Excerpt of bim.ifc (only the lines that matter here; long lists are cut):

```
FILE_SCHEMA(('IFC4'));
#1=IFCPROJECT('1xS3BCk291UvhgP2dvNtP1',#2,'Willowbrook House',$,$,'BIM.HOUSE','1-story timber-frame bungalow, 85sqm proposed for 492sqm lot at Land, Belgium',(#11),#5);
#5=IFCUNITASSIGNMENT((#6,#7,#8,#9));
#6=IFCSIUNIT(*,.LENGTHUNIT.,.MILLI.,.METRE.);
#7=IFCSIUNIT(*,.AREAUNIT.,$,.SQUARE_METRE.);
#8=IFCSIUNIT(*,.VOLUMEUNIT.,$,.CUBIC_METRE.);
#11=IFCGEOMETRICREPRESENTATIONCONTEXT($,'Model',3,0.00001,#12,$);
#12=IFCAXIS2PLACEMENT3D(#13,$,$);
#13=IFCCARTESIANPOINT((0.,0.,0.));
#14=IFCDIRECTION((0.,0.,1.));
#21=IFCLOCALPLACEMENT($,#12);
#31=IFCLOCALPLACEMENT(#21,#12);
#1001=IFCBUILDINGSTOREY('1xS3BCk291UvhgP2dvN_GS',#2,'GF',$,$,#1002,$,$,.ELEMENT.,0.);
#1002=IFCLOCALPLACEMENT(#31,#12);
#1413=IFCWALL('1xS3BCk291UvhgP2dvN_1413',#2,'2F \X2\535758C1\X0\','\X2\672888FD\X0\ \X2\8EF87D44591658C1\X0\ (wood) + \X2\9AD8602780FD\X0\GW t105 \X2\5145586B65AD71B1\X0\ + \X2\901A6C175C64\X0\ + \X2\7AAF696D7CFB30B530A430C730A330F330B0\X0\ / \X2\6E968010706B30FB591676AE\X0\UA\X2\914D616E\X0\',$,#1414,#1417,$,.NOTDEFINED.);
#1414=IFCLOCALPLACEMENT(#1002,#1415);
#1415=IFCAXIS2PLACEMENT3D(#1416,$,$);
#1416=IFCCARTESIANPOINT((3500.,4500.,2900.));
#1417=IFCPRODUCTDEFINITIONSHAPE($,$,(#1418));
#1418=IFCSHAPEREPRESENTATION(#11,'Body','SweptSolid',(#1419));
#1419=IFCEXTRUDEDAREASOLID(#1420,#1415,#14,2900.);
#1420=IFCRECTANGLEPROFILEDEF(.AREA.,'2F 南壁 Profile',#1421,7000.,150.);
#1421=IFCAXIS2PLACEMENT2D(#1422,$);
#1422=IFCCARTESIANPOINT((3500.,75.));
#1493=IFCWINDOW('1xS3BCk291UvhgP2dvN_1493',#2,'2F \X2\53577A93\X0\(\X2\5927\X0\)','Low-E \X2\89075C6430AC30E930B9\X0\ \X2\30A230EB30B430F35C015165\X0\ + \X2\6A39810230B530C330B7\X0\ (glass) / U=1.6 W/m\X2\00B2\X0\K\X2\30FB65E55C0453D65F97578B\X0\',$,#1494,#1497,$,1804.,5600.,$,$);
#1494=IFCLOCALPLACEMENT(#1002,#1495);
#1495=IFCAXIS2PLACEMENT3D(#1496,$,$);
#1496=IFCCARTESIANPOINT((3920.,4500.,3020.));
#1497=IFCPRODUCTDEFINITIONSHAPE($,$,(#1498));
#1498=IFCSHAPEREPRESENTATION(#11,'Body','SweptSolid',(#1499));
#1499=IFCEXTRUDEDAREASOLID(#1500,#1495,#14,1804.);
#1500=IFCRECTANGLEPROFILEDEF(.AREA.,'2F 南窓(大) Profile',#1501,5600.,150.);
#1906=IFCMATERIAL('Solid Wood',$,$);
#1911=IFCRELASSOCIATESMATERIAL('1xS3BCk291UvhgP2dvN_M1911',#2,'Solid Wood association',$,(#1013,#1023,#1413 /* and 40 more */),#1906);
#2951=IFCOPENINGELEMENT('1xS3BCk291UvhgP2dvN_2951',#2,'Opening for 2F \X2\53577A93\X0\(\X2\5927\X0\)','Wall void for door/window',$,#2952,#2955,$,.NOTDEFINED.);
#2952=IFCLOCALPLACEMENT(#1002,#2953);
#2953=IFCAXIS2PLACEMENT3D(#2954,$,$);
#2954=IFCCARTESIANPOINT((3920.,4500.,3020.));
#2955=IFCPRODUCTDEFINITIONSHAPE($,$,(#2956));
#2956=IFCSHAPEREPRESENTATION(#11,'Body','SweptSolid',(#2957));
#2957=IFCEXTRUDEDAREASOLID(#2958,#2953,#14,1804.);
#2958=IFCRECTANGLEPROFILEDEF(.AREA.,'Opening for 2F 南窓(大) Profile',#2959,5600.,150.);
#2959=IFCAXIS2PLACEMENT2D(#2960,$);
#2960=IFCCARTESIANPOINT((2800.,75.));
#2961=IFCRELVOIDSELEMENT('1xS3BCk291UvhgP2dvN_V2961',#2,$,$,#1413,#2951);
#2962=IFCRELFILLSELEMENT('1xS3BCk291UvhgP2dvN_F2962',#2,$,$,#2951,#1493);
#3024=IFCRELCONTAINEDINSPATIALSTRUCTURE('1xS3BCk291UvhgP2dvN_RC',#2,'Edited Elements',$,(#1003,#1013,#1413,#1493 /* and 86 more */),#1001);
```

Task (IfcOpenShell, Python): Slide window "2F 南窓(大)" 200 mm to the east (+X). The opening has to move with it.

```python
import ifcopenshell
import ifcopenshell.api.geometry
import ifcopenshell.util.placement
import ifcopenshell.util.unit

model = ifcopenshell.open("bim.ifc")
unit_scale = ifcopenshell.util.unit.calculate_unit_scale(model)

window = model.by_guid("1xS3BCk291UvhgP2dvN_1493")
opening = window.FillsVoids[0].RelatingOpeningElement
wall = opening.VoidsElements[0].RelatingBuildingElement

wall_matrix = ifcopenshell.util.placement.get_local_placement(wall.ObjectPlacement)
shift = wall_matrix[:3, 0] * 0.2 / unit_scale
before = ifcopenshell.util.placement.get_local_placement(window.ObjectPlacement)[:3, 3].copy()

# The window is not placed relative to its opening, so move both.
for product in (opening, window):
    matrix = ifcopenshell.util.placement.get_local_placement(product.ObjectPlacement)
    matrix[:3, 3] += shift
    ifcopenshell.api.geometry.edit_object_placement(model, product=product, matrix=matrix, is_si=False)

after = ifcopenshell.util.placement.get_local_placement(window.ObjectPlacement)[:3, 3]
print("window moved by", (after - before).round(3) + 0.0)

model.write("bim_rev.ifc")
```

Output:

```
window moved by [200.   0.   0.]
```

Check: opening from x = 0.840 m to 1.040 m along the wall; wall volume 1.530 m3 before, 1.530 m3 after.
